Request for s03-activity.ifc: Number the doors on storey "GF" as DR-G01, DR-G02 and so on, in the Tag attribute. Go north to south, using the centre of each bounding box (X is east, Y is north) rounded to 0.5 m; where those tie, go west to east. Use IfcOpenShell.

First a look at what the model holds.

```python
import ifcopenshell
import ifcopenshell.util.element
import ifcopenshell.util.placement

model = ifcopenshell.open("s03-activity.ifc")
print(model.schema)
storey = next(s for s in model.by_type("IfcBuildingStorey") if s.Name == "GF")
doors = [e for e in ifcopenshell.util.element.get_decomposition(storey) if e.is_a("IfcDoor")]
for e in sorted(doors, key=lambda e: e.id()):
    origin = ifcopenshell.util.placement.get_local_placement(e.ObjectPlacement)[:3, 3]
    print(e.id(), e.Tag, e.Name, origin.round(2) + 0.0, sep=" | ")
```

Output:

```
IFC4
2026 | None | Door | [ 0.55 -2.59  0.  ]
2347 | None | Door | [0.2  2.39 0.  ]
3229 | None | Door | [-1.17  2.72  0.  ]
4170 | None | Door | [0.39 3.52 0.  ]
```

```python
import ifcopenshell
import ifcopenshell.geom
import ifcopenshell.util.element
import ifcopenshell.util.shape

model = ifcopenshell.open("s03-activity.ifc")
settings = ifcopenshell.geom.settings()
settings.set("use-world-coords", True)


def centre(element):
    shape = ifcopenshell.geom.create_shape(settings, element)
    return ifcopenshell.util.shape.get_bbox_centroid(shape.geometry)


storey = next(s for s in model.by_type("IfcBuildingStorey") if s.Name == "GF")
doors = [e for e in ifcopenshell.util.element.get_decomposition(storey) if e.is_a("IfcDoor")]

# Insertion points can sit at a corner or the storey origin, so sort by the geometry (in metres).
centres = {e: centre(e) for e in doors}
doors.sort(key=lambda e: (-round(centres[e][1] / 0.5), centres[e][0]))

for i, e in enumerate(doors, start=1):
    number = f"DR-G{i:02d}"
    e.Tag = number
    print(e.id(), number)

model.write("s03-activity_edited.ifc")
```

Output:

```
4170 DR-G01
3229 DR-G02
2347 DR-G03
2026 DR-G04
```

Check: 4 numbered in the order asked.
